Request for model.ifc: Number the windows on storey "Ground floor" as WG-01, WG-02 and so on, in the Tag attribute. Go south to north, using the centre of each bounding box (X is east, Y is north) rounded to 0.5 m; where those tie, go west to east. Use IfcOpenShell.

First a look at what the model holds.

```python
import ifcopenshell
import ifcopenshell.util.element
import ifcopenshell.util.placement

model = ifcopenshell.open("model.ifc")
print(model.schema)
storey = next(s for s in model.by_type("IfcBuildingStorey") if s.Name == "Ground floor")
windows = [e for e in ifcopenshell.util.element.get_decomposition(storey) if e.is_a("IfcWindow")]
for e in sorted(windows, key=lambda e: e.id()):
    origin = ifcopenshell.util.placement.get_local_placement(e.ObjectPlacement)[:3, 3]
    print(e.id(), e.Tag, e.Name, origin.round(2) + 0.0, sep=" | ")
```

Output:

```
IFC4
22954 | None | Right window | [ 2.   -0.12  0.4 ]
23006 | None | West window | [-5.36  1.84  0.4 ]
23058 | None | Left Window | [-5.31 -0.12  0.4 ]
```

```python
import ifcopenshell
import ifcopenshell.geom
import ifcopenshell.util.element
import ifcopenshell.util.shape

model = ifcopenshell.open("model.ifc")
settings = ifcopenshell.geom.settings()
settings.set("use-world-coords", True)


def centre(element):
    shape = ifcopenshell.geom.create_shape(settings, element)
    return ifcopenshell.util.shape.get_bbox_centroid(shape.geometry)


storey = next(s for s in model.by_type("IfcBuildingStorey") if s.Name == "Ground floor")
windows = [e for e in ifcopenshell.util.element.get_decomposition(storey) if e.is_a("IfcWindow")]

# Insertion points can sit at a corner or the storey origin, so sort by the geometry (in metres).
centres = {e: centre(e) for e in windows}
windows.sort(key=lambda e: (round(centres[e][1] / 0.5), centres[e][0]))

for i, e in enumerate(windows, start=1):
    number = f"WG-{i:02d}"
    e.Tag = number
    print(e.id(), number)

model.write("model_v2.ifc")
```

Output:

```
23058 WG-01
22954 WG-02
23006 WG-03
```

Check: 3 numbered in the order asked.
